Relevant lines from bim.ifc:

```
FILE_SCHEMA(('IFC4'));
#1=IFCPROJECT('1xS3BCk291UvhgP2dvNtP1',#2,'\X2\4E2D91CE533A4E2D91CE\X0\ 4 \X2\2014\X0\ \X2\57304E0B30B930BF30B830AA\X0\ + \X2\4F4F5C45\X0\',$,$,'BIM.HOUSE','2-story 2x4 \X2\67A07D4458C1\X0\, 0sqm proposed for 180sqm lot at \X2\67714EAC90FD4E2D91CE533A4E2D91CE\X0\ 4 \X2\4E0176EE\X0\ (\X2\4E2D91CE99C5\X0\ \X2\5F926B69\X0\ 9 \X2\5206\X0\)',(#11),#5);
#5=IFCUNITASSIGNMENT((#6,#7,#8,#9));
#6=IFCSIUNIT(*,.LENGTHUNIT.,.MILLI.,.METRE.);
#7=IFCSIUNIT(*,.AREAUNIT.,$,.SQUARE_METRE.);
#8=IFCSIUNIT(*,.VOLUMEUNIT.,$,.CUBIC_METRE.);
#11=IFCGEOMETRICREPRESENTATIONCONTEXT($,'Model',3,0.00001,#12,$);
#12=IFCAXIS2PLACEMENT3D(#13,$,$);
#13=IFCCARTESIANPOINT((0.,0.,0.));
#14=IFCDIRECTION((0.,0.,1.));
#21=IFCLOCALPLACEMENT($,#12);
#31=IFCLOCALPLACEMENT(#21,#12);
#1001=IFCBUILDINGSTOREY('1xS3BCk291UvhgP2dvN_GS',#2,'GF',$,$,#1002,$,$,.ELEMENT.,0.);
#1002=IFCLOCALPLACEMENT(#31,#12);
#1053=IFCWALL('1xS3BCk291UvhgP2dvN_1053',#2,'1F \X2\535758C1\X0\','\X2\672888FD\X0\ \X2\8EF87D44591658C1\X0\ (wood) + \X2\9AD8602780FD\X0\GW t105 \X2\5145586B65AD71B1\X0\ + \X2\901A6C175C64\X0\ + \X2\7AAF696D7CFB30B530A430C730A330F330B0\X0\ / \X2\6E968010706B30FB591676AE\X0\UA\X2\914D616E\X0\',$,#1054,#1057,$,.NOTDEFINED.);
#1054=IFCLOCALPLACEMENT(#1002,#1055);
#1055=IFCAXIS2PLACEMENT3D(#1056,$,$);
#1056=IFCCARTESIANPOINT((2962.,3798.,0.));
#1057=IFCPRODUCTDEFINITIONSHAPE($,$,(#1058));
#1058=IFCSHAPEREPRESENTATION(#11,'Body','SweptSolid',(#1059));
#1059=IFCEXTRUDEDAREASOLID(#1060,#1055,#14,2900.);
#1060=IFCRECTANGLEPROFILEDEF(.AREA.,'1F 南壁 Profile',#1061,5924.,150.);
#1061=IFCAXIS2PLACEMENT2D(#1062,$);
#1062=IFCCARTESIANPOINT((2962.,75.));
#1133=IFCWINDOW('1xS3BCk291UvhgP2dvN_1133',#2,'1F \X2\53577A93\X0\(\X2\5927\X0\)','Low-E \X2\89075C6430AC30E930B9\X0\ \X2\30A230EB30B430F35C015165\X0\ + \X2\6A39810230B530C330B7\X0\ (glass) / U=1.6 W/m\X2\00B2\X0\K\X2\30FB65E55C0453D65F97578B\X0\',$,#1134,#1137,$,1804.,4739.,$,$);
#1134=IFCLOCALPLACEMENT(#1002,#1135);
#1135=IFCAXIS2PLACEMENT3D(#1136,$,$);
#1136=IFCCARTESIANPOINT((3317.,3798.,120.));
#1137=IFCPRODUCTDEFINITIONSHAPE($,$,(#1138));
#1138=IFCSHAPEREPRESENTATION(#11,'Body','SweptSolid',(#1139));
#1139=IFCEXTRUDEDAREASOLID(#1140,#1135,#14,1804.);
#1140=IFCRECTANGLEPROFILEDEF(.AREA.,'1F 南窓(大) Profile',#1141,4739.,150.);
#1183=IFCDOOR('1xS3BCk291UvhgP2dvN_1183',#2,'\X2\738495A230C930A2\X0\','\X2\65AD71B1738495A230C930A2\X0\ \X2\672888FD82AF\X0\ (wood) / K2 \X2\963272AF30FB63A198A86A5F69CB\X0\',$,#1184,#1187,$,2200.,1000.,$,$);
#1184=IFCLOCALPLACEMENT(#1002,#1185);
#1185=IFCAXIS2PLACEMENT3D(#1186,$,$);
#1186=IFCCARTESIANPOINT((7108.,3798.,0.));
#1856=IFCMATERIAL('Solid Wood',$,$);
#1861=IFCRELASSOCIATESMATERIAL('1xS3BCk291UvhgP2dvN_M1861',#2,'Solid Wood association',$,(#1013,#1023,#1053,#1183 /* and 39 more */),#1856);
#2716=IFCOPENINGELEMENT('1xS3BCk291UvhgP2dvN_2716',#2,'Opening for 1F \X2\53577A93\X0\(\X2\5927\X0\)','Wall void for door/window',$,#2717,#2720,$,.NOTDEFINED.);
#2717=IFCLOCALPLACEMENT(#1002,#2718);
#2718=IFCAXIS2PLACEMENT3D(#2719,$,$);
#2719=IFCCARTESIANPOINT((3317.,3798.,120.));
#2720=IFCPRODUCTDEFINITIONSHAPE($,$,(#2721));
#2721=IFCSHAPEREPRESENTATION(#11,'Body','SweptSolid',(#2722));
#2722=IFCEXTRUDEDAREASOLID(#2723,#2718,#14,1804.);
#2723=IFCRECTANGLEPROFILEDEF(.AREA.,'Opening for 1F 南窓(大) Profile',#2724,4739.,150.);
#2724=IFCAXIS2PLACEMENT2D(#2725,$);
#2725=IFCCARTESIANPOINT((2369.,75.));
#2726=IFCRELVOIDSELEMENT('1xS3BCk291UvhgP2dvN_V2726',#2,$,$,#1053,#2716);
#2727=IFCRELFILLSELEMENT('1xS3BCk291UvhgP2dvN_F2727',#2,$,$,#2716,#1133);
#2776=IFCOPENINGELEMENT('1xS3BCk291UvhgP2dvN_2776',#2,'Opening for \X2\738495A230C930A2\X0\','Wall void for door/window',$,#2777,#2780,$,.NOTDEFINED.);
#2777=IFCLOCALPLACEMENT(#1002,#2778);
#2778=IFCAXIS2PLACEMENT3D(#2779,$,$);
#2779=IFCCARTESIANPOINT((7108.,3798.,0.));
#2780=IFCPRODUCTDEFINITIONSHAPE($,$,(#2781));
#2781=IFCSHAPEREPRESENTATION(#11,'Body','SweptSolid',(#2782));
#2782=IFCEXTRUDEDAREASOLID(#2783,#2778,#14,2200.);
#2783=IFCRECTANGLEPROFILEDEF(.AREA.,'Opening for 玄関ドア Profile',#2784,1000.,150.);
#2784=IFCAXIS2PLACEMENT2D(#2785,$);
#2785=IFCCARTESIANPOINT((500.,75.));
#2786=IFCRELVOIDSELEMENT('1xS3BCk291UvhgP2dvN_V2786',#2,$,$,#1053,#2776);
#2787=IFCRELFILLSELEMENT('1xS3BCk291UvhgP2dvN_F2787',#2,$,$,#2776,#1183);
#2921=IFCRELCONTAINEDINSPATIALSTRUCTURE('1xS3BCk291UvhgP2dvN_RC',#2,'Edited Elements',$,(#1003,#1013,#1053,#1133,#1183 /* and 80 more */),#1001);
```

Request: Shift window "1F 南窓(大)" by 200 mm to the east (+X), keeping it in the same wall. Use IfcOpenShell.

```python
import ifcopenshell
import ifcopenshell.api.geometry
import ifcopenshell.util.placement
import ifcopenshell.util.unit

model = ifcopenshell.open("bim.ifc")
unit_scale = ifcopenshell.util.unit.calculate_unit_scale(model)

window = model.by_id(1133)
opening = window.FillsVoids[0].RelatingOpeningElement
wall = opening.VoidsElements[0].RelatingBuildingElement

wall_matrix = ifcopenshell.util.placement.get_local_placement(wall.ObjectPlacement)
shift = wall_matrix[:3, 0] * 0.2 / unit_scale
before = ifcopenshell.util.placement.get_local_placement(window.ObjectPlacement)[:3, 3].copy()

# The window is not placed relative to its opening, so move both.
for product in (opening, window):
    matrix = ifcopenshell.util.placement.get_local_placement(product.ObjectPlacement)
    matrix[:3, 3] += shift
    ifcopenshell.api.geometry.edit_object_placement(model, product=product, matrix=matrix, is_si=False)

after = ifcopenshell.util.placement.get_local_placement(window.ObjectPlacement)[:3, 3]
print("window moved by", (after - before).round(3) + 0.0)

model.write("bim_edited.ifc")
```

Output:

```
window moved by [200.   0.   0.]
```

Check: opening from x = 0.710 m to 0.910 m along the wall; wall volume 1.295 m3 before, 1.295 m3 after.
